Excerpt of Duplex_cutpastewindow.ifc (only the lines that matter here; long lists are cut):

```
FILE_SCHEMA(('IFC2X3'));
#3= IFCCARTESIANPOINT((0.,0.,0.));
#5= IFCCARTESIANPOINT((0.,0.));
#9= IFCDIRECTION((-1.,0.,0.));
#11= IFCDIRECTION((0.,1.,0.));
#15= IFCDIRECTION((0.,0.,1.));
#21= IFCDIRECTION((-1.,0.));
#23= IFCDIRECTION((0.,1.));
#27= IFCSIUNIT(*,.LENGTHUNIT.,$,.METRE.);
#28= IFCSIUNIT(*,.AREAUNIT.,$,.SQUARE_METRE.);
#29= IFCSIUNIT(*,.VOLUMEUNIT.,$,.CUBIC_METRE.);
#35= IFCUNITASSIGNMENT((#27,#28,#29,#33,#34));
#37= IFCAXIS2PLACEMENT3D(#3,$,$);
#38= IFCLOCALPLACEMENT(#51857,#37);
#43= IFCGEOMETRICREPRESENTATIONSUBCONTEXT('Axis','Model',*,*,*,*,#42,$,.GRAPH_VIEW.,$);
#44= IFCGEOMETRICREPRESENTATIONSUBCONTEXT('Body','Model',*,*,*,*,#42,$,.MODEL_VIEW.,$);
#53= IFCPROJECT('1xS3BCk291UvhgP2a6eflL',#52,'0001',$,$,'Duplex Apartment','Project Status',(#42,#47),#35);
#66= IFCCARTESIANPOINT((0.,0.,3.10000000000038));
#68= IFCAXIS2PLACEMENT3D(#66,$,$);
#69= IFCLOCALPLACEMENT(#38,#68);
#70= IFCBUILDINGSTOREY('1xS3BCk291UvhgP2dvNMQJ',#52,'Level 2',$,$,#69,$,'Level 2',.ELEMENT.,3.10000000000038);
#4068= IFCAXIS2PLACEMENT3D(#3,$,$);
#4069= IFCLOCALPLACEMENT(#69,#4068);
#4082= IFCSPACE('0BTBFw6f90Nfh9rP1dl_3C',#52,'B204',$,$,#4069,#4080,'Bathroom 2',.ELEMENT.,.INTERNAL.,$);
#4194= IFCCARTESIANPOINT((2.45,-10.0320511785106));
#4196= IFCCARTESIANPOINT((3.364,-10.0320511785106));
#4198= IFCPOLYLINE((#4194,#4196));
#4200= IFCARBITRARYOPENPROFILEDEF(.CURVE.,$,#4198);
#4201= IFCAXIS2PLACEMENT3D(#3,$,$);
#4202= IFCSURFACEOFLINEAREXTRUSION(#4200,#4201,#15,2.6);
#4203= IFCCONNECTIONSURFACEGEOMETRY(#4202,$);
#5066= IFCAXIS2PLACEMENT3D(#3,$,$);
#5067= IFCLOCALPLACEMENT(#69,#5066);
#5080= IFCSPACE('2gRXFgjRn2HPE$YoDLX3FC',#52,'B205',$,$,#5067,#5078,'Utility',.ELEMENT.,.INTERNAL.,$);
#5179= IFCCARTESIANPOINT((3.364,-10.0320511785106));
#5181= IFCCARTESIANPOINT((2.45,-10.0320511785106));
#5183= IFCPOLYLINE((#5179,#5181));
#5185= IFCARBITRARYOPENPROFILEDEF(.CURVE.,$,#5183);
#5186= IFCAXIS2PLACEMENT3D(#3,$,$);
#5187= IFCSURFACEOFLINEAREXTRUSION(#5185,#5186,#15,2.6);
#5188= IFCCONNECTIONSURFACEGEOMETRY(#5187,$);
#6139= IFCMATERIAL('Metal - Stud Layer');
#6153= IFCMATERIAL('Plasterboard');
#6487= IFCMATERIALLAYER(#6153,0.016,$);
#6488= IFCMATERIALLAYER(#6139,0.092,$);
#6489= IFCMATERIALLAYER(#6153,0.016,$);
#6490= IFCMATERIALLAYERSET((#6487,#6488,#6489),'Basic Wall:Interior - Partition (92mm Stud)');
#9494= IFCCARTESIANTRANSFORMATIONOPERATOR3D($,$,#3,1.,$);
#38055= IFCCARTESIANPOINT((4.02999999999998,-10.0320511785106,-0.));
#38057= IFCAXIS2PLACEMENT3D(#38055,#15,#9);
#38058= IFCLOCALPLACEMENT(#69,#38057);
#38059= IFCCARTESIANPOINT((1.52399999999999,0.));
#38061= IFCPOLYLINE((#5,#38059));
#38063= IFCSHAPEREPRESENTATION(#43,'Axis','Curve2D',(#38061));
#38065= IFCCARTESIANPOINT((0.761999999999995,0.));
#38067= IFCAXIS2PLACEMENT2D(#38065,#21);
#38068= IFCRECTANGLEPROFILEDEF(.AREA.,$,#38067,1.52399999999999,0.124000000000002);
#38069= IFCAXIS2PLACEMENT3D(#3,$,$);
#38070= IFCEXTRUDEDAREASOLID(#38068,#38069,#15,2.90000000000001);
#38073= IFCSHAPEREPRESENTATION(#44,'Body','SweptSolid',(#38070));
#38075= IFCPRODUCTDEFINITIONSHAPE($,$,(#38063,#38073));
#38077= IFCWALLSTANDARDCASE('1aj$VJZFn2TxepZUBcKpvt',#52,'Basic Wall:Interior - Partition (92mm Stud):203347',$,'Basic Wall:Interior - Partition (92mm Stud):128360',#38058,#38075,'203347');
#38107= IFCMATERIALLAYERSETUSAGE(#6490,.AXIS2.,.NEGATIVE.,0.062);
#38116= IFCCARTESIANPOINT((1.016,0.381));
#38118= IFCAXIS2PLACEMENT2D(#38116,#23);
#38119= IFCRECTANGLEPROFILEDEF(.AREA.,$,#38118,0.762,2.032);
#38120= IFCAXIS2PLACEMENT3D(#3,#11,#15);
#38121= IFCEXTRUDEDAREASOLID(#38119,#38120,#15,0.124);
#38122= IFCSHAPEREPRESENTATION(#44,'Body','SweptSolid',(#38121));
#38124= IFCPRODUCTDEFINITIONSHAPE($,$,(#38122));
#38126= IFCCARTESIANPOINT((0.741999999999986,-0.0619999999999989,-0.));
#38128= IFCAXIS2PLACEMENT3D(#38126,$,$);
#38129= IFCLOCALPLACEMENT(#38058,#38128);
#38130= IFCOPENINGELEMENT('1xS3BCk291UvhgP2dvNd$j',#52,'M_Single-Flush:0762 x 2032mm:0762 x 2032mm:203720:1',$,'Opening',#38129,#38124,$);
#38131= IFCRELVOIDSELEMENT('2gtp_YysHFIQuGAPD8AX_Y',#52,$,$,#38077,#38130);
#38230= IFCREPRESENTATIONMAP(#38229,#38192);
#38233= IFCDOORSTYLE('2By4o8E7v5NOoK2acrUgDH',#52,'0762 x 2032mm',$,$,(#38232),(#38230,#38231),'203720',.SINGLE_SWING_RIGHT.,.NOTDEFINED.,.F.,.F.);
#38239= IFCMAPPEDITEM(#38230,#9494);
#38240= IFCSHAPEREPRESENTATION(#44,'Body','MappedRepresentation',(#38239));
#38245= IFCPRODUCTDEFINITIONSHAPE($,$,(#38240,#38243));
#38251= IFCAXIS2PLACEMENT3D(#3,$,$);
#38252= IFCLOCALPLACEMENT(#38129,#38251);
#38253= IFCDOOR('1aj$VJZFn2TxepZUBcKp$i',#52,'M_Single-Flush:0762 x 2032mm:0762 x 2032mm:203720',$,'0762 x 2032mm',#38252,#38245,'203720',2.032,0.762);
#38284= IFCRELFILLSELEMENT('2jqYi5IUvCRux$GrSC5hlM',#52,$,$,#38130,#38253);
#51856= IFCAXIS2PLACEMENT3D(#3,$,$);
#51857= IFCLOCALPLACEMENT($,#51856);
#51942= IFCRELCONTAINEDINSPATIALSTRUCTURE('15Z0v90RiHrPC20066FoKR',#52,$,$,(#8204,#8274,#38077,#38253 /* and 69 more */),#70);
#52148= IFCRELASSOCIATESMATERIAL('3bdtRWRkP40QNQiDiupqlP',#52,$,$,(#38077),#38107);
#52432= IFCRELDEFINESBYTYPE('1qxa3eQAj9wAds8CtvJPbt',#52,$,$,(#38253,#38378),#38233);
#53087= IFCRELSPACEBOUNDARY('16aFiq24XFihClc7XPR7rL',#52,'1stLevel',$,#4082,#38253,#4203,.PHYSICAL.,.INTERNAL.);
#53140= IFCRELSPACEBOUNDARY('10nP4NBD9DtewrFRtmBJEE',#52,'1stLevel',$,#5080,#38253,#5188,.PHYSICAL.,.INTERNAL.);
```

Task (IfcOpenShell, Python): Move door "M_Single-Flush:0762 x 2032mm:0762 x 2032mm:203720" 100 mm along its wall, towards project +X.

```python
import numpy as np
import ifcopenshell
import ifcopenshell.api.geometry
import ifcopenshell.util.placement
import ifcopenshell.util.unit

model = ifcopenshell.open("Duplex_cutpastewindow.ifc")
unit_scale = ifcopenshell.util.unit.calculate_unit_scale(model)

door = model.by_id(38253)
opening = door.FillsVoids[0].RelatingOpeningElement
wall = opening.VoidsElements[0].RelatingBuildingElement

wall_matrix = ifcopenshell.util.placement.get_local_placement(wall.ObjectPlacement)
shift = wall_matrix[:3, 0] * -0.1 / unit_scale
before = ifcopenshell.util.placement.get_local_placement(door.ObjectPlacement)[:3, 3].copy()

# The door is placed relative to its opening, so it follows when the opening moves.
matrix = ifcopenshell.util.placement.get_local_placement(opening.ObjectPlacement)
matrix[:3, 3] += shift
ifcopenshell.api.geometry.edit_object_placement(
    model, product=opening, matrix=matrix, is_si=False, should_transform_children=True
)

# Space boundary surfaces are stored in each space's coordinates; move them too.
for rel in door.ProvidesBoundaries:
    if not rel.ConnectionGeometry:
        continue
    surface = rel.ConnectionGeometry.SurfaceOnRelatingElement
    space_matrix = ifcopenshell.util.placement.get_local_placement(rel.RelatingSpace.ObjectPlacement)
    point = np.array(surface.Position.Location.Coordinates) + space_matrix[:3, :3].T @ shift
    surface.Position = model.createIfcAxis2Placement3D(
        model.createIfcCartesianPoint(point.tolist()), surface.Position.Axis, surface.Position.RefDirection
    )

after = ifcopenshell.util.placement.get_local_placement(door.ObjectPlacement)[:3, 3]
print("door moved by", (after - before).round(3) + 0.0)

model.write("Duplex_cutpastewindow-out.ifc")
```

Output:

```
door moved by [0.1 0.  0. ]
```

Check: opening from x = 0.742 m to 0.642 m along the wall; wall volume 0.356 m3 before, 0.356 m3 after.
